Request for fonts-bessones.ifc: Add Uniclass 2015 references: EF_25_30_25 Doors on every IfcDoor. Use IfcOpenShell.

First a look at what the model holds.

```python
import ifcopenshell

model = ifcopenshell.open("fonts-bessones.ifc")
print(model.schema)
print("classifications:", [c.Name for c in model.by_type("IfcClassification")])
for ifc_class in ("IfcDoor", "IfcRoof", "IfcStair", "IfcWall", "IfcWindow"):
    print(ifc_class, len(model.by_type(ifc_class)))
```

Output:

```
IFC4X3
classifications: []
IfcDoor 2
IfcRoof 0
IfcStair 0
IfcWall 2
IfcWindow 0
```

```python
import ifcopenshell
import ifcopenshell.api.classification

model = ifcopenshell.open("fonts-bessones.ifc")

system = ifcopenshell.api.classification.add_classification(model, classification="Uniclass 2015")

codes = {
    "IfcDoor": ("EF_25_30_25", "Doors"),
}
for ifc_class, (code, name) in codes.items():
    products = model.by_type(ifc_class)
    ifcopenshell.api.classification.add_reference(
        model, products=products, classification=system, identification=code, name=name
    )
    print(code, len(products))

model.write("fonts-bessones_edited.ifc")
```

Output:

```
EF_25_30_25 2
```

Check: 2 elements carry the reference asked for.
